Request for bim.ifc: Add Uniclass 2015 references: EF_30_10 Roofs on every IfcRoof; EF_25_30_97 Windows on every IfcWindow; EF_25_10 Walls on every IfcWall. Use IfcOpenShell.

First a look at what the model holds.

```python
import ifcopenshell

model = ifcopenshell.open("bim.ifc")
print(model.schema)
print("classifications:", [c.Name for c in model.by_type("IfcClassification")])
for ifc_class in ("IfcDoor", "IfcRoof", "IfcStair", "IfcWall", "IfcWindow"):
    print(ifc_class, len(model.by_type(ifc_class)))
```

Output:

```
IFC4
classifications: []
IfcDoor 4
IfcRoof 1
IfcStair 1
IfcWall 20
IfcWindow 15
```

```python
import ifcopenshell
import ifcopenshell.api.classification

model = ifcopenshell.open("bim.ifc")

system = ifcopenshell.api.classification.add_classification(model, classification="Uniclass 2015")

codes = {
    "IfcRoof": ("EF_30_10", "Roofs"),
    "IfcWindow": ("EF_25_30_97", "Windows"),
    "IfcWall": ("EF_25_10", "Walls"),
}
for ifc_class, (code, name) in codes.items():
    products = model.by_type(ifc_class)
    ifcopenshell.api.classification.add_reference(
        model, products=products, classification=system, identification=code, name=name
    )
    print(code, len(products))

model.write("bim_rev.ifc")
```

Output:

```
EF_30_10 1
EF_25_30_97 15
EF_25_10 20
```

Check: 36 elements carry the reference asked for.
